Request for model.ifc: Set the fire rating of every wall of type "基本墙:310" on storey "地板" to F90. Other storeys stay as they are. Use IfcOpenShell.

First a look at what the model holds.

```python
import ifcopenshell
import ifcopenshell.util.element

model = ifcopenshell.open("model.ifc")
print(model.schema)
storey = next(s for s in model.by_type("IfcBuildingStorey") if s.Name == "地板")
walls = [e for e in ifcopenshell.util.element.get_decomposition(storey) if e.is_a("IfcWall")]
seen = {}
for e in walls:
    element_type = ifcopenshell.util.element.get_type(e)
    key = (element_type.Name if element_type != e and element_type else None, ifcopenshell.util.element.get_pset(e, "Pset_WallCommon", "FireRating"))
    seen[key] = seen.get(key, 0) + 1
for (name, value), count in sorted(seen.items(), key=str):
    print(count, "x", name, "|", value)
```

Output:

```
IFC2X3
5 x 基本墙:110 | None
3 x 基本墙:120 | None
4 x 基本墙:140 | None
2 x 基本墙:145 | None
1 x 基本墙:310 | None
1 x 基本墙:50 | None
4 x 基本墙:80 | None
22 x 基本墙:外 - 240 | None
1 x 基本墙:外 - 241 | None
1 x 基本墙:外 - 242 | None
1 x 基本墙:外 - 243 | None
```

```python
import ifcopenshell
import ifcopenshell.api.pset
import ifcopenshell.util.element

model = ifcopenshell.open("model.ifc")

storey = next(s for s in model.by_type("IfcBuildingStorey") if s.Name == "地板")
walls = [e for e in ifcopenshell.util.element.get_decomposition(storey) if e.is_a("IfcWall")]

count = 0
for e in walls:
    element_type = ifcopenshell.util.element.get_type(e)
    if element_type in (None, e) or element_type.Name != "基本墙:310":
        continue
    # add_pset returns the element's existing set when there is one.
    pset = ifcopenshell.api.pset.add_pset(model, product=e, name="Pset_WallCommon")
    ifcopenshell.api.pset.edit_pset(model, pset=pset, properties={"FireRating": "F90"})
    count += 1

print(count, "walls updated")

model.write("model-out.ifc")
```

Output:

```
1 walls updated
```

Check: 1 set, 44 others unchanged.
